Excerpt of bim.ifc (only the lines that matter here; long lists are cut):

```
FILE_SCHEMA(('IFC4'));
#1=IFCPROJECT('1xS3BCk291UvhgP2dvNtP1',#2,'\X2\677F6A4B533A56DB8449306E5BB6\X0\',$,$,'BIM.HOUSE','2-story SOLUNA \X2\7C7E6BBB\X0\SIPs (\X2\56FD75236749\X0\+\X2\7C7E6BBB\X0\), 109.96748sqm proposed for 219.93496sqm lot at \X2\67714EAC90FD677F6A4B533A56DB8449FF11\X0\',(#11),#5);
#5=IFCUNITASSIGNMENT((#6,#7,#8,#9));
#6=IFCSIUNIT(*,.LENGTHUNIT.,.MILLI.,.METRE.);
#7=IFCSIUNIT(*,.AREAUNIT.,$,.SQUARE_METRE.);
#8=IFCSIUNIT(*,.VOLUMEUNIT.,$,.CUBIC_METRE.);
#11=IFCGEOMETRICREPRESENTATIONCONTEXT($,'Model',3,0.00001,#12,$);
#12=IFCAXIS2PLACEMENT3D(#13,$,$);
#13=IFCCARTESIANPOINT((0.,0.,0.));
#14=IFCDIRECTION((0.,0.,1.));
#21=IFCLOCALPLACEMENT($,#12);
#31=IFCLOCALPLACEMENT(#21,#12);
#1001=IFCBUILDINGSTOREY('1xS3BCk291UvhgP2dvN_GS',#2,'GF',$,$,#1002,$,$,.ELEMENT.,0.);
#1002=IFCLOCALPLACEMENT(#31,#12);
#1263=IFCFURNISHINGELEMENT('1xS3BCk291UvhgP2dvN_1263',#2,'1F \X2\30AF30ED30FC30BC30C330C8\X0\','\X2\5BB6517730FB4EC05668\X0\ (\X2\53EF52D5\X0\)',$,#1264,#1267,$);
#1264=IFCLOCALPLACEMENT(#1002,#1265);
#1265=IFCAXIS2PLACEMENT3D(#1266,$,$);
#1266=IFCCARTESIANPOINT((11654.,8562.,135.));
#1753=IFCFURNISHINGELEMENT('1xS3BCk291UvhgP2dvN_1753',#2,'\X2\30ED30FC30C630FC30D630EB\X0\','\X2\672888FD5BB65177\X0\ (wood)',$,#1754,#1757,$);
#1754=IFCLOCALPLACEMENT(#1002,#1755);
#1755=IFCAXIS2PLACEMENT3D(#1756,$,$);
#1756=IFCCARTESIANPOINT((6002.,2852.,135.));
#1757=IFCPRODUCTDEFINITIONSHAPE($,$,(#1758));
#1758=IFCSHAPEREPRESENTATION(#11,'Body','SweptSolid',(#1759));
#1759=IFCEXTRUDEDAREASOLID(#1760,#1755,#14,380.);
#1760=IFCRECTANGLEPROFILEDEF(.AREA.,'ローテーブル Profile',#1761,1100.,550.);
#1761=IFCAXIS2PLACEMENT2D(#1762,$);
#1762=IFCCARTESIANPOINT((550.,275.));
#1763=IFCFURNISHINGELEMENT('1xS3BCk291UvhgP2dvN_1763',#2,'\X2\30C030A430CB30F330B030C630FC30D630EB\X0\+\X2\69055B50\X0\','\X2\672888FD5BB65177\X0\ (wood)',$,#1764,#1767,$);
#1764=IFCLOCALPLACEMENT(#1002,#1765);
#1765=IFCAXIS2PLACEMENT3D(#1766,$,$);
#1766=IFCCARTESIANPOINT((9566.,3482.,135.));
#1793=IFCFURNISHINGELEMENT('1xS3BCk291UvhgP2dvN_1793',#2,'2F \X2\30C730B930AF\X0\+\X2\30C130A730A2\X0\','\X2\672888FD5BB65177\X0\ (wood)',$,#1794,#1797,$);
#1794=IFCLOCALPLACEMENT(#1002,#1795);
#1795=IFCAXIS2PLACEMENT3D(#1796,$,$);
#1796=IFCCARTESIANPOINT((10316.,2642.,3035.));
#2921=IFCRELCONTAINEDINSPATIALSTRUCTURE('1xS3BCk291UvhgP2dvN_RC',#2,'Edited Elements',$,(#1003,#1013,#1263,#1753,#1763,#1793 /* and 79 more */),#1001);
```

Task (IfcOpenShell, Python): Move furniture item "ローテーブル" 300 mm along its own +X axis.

```python
import ifcopenshell
import ifcopenshell.api.geometry
import ifcopenshell.util.placement
import ifcopenshell.util.unit

model = ifcopenshell.open("bim.ifc")
unit_scale = ifcopenshell.util.unit.calculate_unit_scale(model)

item = model.by_id(1753)
matrix = ifcopenshell.util.placement.get_local_placement(item.ObjectPlacement)
matrix[:3, 3] += matrix[:3, 0] * 0.3 / unit_scale
ifcopenshell.api.geometry.edit_object_placement(model, product=item, matrix=matrix, is_si=False)

print(ifcopenshell.util.placement.get_local_placement(item.ObjectPlacement).round(3) + 0.0)

model.write("bim-out.ifc")
```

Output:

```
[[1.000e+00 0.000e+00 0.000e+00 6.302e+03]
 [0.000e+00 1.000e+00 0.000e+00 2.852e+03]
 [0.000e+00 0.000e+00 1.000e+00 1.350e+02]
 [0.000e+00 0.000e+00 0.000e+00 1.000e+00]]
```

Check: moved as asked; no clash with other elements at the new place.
